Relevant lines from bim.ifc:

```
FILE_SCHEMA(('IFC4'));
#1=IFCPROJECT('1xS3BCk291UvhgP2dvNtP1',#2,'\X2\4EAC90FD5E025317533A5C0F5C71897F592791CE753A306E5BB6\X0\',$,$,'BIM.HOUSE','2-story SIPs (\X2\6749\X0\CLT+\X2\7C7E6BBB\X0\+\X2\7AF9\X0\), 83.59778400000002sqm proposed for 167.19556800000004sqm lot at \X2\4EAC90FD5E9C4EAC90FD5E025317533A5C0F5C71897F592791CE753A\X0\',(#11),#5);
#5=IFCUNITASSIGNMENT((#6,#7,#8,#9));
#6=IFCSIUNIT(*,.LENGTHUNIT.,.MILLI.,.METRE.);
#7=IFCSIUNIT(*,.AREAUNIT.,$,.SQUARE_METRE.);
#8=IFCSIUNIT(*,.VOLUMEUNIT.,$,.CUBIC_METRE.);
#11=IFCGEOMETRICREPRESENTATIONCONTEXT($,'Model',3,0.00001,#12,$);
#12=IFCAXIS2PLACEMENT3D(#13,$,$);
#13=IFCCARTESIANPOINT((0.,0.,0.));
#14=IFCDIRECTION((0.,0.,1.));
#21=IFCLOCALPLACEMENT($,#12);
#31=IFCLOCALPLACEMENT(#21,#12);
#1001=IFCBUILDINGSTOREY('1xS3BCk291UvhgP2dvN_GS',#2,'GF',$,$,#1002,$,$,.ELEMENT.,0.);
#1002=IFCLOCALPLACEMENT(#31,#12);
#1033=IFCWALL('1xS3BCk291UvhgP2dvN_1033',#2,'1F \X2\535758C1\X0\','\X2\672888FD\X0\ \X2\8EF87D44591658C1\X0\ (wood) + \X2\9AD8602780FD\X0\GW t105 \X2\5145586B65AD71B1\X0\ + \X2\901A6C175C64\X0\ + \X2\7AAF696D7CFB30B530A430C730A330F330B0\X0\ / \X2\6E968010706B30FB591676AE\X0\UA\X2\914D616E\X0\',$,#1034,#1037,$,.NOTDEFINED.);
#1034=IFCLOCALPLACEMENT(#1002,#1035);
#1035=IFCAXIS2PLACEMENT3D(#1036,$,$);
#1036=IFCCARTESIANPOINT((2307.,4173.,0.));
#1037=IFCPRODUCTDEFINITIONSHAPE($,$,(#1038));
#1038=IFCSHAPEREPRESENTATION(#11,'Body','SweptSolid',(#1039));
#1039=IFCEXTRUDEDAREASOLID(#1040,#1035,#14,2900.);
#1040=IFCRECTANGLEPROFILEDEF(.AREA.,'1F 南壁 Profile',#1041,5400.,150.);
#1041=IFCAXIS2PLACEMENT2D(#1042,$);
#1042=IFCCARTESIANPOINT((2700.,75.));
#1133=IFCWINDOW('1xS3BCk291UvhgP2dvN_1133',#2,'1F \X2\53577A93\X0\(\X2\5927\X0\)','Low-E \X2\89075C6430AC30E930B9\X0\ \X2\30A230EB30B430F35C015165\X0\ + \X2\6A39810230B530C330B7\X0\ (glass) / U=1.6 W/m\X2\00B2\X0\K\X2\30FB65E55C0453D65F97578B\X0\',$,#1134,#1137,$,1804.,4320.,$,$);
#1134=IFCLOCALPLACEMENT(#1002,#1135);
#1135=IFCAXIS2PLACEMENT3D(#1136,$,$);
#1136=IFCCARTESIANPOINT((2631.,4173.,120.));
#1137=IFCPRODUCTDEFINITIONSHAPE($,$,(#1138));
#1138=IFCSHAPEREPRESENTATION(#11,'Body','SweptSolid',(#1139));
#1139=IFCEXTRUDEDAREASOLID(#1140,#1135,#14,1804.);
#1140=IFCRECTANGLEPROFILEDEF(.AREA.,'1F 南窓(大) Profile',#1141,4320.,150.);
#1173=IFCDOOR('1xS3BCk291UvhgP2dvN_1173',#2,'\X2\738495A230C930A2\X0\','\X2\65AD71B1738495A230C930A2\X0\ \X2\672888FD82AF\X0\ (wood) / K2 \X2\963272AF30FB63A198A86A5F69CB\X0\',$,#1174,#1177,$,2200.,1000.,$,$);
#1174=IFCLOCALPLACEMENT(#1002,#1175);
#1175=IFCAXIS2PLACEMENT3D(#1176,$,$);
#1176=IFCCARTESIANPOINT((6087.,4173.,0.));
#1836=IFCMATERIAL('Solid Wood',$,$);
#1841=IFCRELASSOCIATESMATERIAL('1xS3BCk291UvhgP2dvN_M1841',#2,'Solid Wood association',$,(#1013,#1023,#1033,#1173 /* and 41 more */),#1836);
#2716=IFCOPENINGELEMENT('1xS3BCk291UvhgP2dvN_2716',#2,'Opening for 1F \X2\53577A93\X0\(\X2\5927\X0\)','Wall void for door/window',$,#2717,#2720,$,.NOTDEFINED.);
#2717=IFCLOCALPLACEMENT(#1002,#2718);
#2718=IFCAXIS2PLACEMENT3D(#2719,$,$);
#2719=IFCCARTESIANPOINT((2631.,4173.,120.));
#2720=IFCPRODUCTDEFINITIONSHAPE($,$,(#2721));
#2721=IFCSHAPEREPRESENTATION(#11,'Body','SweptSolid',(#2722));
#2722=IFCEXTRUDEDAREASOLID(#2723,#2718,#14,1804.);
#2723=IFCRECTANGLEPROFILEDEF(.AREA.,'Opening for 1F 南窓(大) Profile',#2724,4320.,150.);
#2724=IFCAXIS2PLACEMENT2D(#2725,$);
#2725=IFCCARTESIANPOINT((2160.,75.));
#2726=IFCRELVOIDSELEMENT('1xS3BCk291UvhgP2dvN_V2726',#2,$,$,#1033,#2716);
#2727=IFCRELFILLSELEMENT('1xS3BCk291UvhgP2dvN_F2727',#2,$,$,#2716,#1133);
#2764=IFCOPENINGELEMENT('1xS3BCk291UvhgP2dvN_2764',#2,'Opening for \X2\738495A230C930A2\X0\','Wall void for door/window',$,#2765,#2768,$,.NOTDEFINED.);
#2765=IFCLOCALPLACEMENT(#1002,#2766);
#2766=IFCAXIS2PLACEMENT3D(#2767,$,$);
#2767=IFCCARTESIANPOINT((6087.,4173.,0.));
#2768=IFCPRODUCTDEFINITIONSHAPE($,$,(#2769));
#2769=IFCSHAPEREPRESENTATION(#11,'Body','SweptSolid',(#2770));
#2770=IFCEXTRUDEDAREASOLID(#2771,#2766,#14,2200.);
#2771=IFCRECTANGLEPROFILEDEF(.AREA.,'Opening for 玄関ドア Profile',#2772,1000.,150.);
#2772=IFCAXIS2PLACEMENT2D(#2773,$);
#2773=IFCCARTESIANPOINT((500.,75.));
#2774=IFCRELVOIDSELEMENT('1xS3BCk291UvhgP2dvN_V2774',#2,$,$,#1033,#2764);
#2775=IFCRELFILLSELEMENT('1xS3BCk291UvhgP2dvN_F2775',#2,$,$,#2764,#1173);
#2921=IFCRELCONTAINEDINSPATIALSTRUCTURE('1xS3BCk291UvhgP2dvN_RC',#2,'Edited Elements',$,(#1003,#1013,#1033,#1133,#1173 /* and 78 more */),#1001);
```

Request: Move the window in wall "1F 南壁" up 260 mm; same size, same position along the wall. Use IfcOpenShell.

```python
import numpy as np
import ifcopenshell
import ifcopenshell.api.geometry
import ifcopenshell.util.placement
import ifcopenshell.util.unit

model = ifcopenshell.open("bim.ifc")
unit_scale = ifcopenshell.util.unit.calculate_unit_scale(model)

window = model.by_guid("1xS3BCk291UvhgP2dvN_1133")
opening = window.FillsVoids[0].RelatingOpeningElement
dz = 0.26 / unit_scale

shift = np.array([0.0, 0.0, dz])
# The window is not placed relative to its opening, so move both.
for product in (opening, window):
    matrix = ifcopenshell.util.placement.get_local_placement(product.ObjectPlacement)
    matrix[:3, 3] += shift
    ifcopenshell.api.geometry.edit_object_placement(model, product=product, matrix=matrix, is_si=False)

print(f"moved by {dz * unit_scale:+.3f} m")

model.write("bim_updated.ifc")
```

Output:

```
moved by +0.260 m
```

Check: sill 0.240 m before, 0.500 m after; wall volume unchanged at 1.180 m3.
